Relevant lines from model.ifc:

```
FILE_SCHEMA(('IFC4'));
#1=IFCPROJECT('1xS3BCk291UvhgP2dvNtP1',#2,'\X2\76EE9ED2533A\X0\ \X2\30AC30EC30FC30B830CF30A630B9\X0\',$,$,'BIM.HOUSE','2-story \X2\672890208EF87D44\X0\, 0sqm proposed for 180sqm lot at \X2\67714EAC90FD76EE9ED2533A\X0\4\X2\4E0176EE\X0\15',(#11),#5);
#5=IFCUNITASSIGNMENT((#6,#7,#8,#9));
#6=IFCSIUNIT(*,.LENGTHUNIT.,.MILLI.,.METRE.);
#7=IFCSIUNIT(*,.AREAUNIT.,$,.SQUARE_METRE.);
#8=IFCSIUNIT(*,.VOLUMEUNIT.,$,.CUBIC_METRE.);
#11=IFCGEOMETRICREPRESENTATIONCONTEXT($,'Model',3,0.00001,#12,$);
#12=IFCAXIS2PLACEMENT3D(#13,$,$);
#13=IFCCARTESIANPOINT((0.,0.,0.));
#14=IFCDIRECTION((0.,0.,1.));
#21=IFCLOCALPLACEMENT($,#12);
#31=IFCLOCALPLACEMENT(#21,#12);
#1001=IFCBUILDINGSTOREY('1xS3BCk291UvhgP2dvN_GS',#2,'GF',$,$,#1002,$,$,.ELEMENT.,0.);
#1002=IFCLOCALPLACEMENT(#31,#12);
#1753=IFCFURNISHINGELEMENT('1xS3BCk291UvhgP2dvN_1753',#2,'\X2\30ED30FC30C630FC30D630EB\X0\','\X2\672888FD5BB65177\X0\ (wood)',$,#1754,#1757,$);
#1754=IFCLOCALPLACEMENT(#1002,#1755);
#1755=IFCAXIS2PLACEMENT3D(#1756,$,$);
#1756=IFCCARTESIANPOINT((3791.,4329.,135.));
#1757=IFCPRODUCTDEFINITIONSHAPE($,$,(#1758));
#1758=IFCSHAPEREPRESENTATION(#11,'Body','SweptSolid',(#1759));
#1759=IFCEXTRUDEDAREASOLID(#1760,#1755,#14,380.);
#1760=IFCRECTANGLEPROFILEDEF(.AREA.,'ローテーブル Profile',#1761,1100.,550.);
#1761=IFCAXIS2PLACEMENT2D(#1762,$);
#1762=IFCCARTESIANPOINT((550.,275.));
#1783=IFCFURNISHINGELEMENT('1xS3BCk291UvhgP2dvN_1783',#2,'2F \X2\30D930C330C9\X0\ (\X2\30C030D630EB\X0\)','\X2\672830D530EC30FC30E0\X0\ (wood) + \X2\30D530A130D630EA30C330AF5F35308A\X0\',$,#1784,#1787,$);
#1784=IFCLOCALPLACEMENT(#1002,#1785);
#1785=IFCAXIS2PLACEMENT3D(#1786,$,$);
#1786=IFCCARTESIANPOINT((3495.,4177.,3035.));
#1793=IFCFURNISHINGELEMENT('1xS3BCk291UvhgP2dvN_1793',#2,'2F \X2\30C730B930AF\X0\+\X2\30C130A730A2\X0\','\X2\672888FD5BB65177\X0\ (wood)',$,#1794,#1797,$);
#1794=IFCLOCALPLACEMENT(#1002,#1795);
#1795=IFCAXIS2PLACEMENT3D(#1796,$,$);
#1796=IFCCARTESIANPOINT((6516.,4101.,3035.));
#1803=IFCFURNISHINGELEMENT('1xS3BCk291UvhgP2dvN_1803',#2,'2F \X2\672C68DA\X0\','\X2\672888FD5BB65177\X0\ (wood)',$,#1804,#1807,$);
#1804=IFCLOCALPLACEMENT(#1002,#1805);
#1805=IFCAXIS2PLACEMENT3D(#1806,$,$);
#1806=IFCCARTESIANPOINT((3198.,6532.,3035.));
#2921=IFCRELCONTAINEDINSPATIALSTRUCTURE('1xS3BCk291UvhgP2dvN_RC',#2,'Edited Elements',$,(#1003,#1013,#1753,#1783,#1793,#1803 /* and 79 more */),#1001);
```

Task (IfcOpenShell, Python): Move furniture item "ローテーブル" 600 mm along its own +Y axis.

```python
import ifcopenshell
import ifcopenshell.api.geometry
import ifcopenshell.util.placement
import ifcopenshell.util.unit

model = ifcopenshell.open("model.ifc")
unit_scale = ifcopenshell.util.unit.calculate_unit_scale(model)

item = model.by_guid("1xS3BCk291UvhgP2dvN_1753")
matrix = ifcopenshell.util.placement.get_local_placement(item.ObjectPlacement)
matrix[:3, 3] += matrix[:3, 1] * 0.6 / unit_scale
ifcopenshell.api.geometry.edit_object_placement(model, product=item, matrix=matrix, is_si=False)

print(ifcopenshell.util.placement.get_local_placement(item.ObjectPlacement).round(3) + 0.0)

model.write("model-out.ifc")
```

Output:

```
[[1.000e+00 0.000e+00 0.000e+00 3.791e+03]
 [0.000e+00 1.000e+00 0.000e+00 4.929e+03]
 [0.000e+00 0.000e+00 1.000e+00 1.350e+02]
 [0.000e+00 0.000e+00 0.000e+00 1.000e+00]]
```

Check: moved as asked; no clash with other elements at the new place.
